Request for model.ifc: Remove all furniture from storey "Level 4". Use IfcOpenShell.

First a look at what the model holds.

```python
import ifcopenshell
import ifcopenshell.util.element

model = ifcopenshell.open("model.ifc")
print(model.schema)
storey = next(s for s in model.by_type("IfcBuildingStorey") if s.Name == "Level 4")
furniture = [e for e in ifcopenshell.util.element.get_decomposition(storey) if e.is_a("IfcFurnishingElement")]
seen = {}
for e in furniture:
    element_type = ifcopenshell.util.element.get_type(e)
    name = element_type.Name if element_type not in (None, e) else None
    seen[name] = seen.get(name, 0) + 1
for name, count in sorted(seen.items(), key=str):
    print(count, "x", name)
```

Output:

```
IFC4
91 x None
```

```python
import ifcopenshell
import ifcopenshell.api.root
import ifcopenshell.util.element

model = ifcopenshell.open("model.ifc")

storey = next(s for s in model.by_type("IfcBuildingStorey") if s.Name == "Level 4")
furniture = [e for e in ifcopenshell.util.element.get_decomposition(storey) if e.is_a("IfcFurnishingElement")]

for e in furniture:
    ifcopenshell.api.root.remove_product(model, product=e)
print(len(furniture), "removed")

model.write("model_v2.ifc")
```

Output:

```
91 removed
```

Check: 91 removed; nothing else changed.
